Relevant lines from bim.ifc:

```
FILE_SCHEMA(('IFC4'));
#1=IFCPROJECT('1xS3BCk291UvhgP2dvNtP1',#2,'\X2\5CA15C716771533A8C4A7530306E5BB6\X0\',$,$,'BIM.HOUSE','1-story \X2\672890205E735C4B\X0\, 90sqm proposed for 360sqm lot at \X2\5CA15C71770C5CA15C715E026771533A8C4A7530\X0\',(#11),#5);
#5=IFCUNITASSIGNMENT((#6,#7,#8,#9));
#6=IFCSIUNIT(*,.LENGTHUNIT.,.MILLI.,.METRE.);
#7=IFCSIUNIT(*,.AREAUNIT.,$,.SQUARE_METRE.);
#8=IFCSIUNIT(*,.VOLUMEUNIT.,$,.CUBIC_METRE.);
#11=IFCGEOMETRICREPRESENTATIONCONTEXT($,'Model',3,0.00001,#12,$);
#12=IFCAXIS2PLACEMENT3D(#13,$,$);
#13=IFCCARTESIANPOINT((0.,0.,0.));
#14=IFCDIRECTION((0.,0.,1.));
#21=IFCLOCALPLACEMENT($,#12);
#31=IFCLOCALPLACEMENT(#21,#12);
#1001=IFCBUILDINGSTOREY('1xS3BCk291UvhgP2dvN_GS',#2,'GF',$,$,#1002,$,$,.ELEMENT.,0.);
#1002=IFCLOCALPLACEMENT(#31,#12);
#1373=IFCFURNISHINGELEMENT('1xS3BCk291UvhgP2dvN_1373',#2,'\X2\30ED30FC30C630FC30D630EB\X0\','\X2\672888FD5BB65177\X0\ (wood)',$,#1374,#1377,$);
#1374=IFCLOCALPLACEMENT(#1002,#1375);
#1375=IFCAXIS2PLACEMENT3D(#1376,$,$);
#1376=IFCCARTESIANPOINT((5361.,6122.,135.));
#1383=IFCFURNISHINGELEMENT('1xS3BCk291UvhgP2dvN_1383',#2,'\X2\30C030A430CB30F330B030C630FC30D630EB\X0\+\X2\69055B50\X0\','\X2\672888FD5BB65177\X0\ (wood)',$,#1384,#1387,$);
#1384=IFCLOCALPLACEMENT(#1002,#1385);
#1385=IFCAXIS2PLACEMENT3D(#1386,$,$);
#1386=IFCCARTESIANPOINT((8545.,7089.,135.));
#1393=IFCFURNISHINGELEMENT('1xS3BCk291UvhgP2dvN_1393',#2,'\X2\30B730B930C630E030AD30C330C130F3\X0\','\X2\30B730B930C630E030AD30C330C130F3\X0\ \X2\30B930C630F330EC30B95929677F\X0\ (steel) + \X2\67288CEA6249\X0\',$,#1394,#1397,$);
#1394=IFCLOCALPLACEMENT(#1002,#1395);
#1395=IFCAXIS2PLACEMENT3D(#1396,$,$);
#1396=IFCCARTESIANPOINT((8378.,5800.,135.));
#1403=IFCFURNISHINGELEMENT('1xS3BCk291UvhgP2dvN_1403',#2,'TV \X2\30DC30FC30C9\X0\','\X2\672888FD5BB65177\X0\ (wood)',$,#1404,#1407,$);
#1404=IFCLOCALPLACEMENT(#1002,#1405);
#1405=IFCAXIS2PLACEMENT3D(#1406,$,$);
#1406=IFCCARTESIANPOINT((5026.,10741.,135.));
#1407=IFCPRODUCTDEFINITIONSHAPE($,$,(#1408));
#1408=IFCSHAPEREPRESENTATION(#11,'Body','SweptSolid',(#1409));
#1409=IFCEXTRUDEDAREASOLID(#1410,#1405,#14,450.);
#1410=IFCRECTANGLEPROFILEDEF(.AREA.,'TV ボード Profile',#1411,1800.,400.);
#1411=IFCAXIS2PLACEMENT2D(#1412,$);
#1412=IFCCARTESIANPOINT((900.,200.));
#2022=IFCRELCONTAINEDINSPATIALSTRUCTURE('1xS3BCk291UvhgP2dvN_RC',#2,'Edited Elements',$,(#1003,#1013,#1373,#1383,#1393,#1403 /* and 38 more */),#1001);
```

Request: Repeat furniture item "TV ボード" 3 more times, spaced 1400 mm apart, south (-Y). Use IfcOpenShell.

```python
import numpy as np
import ifcopenshell
import ifcopenshell.api.geometry
import ifcopenshell.api.root
import ifcopenshell.util.element
import ifcopenshell.util.placement

model = ifcopenshell.open("bim.ifc")


def reuse_history(source, copy):
    """copy_class also copies each property set's owner history, people and application; keep the originals."""
    for rel in copy.IsDefinedBy:
        if rel.is_a("IfcRelDefinesByProperties") and (history := rel.RelatingPropertyDefinition.OwnerHistory):
            rel.RelatingPropertyDefinition.OwnerHistory = source.OwnerHistory
            ifcopenshell.util.element.remove_deep2(model, history)


source = model.by_guid("1xS3BCk291UvhgP2dvN_1403")
base = ifcopenshell.util.placement.get_local_placement(source.ObjectPlacement)
step = np.array([0.0, -1.0, 0.0]) * 1400.0

for i in range(1, 4):
    copy = ifcopenshell.api.root.copy_class(model, product=source)
    copy.Representation = ifcopenshell.util.element.copy_deep(
        model, source.Representation, exclude=["IfcGeometricRepresentationContext", "IfcRepresentationMap"]
    )
    reuse_history(source, copy)
    matrix = base.copy()
    matrix[:3, 3] += i * step
    print("added at", matrix[:3, 3].round(3) + 0.0)
    ifcopenshell.api.geometry.edit_object_placement(model, product=copy, matrix=matrix, is_si=False)

model.write("bim_v2.ifc")
```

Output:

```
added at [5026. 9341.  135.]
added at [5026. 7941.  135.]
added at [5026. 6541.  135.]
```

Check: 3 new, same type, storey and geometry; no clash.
